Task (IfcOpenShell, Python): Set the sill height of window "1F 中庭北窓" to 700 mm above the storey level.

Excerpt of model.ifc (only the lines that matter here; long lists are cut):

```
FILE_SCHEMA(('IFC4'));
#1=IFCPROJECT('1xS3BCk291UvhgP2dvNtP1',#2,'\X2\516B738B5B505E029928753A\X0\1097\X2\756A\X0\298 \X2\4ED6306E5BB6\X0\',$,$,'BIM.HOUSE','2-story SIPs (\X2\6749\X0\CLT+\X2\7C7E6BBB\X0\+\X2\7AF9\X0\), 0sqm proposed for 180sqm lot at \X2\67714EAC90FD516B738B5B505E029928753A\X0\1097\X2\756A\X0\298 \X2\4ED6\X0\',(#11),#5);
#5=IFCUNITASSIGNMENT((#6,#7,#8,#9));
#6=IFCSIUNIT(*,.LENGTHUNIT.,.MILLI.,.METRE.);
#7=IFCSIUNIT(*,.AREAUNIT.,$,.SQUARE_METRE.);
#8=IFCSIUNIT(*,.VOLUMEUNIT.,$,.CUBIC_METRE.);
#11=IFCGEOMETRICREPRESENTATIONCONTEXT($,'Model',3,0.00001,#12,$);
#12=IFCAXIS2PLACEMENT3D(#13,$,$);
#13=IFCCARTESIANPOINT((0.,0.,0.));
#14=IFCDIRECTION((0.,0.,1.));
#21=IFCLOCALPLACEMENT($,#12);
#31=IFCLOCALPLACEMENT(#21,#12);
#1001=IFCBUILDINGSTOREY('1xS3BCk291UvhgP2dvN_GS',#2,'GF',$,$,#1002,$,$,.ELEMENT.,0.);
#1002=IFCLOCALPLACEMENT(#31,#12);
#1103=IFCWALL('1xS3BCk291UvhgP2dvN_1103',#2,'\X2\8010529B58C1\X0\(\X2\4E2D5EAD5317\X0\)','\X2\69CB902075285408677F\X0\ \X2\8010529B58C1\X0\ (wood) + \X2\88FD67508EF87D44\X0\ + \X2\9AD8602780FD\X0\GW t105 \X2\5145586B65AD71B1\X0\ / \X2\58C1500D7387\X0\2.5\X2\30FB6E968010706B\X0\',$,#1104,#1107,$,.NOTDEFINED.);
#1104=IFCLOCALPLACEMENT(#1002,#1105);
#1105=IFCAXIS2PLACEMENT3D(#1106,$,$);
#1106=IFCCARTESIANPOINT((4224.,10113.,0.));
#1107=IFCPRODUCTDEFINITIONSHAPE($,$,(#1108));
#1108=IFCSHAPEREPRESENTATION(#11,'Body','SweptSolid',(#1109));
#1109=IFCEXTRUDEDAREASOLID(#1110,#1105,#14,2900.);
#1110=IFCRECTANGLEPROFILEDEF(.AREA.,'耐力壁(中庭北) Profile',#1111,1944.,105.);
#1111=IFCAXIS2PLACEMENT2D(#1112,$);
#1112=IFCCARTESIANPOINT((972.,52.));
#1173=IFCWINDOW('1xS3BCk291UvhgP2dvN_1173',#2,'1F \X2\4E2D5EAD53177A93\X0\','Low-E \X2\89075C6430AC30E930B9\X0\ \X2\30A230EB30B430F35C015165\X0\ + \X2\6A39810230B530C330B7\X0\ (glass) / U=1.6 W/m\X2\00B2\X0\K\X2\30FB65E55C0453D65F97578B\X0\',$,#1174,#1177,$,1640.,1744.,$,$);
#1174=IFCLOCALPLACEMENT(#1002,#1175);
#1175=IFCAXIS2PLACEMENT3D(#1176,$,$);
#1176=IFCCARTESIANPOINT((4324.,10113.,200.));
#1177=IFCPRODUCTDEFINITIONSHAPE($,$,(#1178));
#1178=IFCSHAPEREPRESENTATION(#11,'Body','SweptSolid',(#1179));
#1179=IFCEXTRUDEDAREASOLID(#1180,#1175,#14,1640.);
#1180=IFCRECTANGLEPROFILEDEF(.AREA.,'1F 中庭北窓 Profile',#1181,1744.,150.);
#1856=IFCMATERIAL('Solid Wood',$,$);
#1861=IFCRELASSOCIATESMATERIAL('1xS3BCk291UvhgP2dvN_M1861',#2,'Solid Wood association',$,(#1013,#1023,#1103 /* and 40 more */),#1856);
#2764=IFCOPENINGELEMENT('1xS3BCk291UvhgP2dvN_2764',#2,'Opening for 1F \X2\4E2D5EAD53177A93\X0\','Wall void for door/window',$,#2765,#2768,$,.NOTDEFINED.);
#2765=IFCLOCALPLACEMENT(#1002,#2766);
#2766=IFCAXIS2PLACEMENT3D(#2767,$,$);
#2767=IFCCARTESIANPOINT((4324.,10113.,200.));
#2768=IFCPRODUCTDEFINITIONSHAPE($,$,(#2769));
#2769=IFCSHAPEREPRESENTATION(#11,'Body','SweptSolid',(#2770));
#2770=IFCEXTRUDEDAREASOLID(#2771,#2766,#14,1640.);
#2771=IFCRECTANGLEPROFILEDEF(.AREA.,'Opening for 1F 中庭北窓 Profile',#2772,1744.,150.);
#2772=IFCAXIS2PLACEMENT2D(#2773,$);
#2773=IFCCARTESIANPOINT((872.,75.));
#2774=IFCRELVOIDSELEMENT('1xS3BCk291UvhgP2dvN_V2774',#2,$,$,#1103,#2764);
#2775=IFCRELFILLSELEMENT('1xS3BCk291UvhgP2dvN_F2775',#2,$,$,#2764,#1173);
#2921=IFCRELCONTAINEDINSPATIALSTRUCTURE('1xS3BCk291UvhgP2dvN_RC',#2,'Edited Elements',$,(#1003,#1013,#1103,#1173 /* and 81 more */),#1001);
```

```python
import numpy as np
import ifcopenshell
import ifcopenshell.api.geometry
import ifcopenshell.geom
import ifcopenshell.util.element
import ifcopenshell.util.placement
import ifcopenshell.util.shape
import ifcopenshell.util.unit

model = ifcopenshell.open("model.ifc")
unit_scale = ifcopenshell.util.unit.calculate_unit_scale(model)

window = model.by_id(1173)
opening = window.FillsVoids[0].RelatingOpeningElement
storey = ifcopenshell.util.element.get_container(window, ifc_class="IfcBuildingStorey")
level = ifcopenshell.util.placement.get_local_placement(storey.ObjectPlacement)[2, 3]

# The opening's origin need not be at the sill, so measure its lowest point.
shape = ifcopenshell.geom.create_shape(ifcopenshell.geom.settings(), opening)
bottom = ifcopenshell.util.shape.get_shape_bottom_elevation(shape, shape.geometry) / unit_scale
dz = level + 700.0 - bottom

shift = np.array([0.0, 0.0, dz])
# The window is not placed relative to its opening, so move both.
for product in (opening, window):
    matrix = ifcopenshell.util.placement.get_local_placement(product.ObjectPlacement)
    matrix[:3, 3] += shift
    ifcopenshell.api.geometry.edit_object_placement(model, product=product, matrix=matrix, is_si=False)

print(f"moved by {dz * unit_scale:+.3f} m")

model.write("model_updated.ifc")
```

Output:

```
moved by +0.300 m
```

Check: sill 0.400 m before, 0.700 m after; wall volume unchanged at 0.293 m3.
